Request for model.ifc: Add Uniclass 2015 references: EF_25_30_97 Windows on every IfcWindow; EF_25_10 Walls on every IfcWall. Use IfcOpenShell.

First a look at what the model holds.

```python
import ifcopenshell

model = ifcopenshell.open("model.ifc")
print(model.schema)
print("classifications:", [c.Name for c in model.by_type("IfcClassification")])
for ifc_class in ("IfcDoor", "IfcRoof", "IfcStair", "IfcWall", "IfcWindow"):
    print(ifc_class, len(model.by_type(ifc_class)))
```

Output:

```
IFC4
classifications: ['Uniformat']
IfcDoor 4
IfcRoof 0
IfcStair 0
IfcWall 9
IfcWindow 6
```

```python
import ifcopenshell
import ifcopenshell.api.classification

model = ifcopenshell.open("model.ifc")

system = ifcopenshell.api.classification.add_classification(model, classification="Uniclass 2015")

codes = {
    "IfcWindow": ("EF_25_30_97", "Windows"),
    "IfcWall": ("EF_25_10", "Walls"),
}
for ifc_class, (code, name) in codes.items():
    products = model.by_type(ifc_class)
    ifcopenshell.api.classification.add_reference(
        model, products=products, classification=system, identification=code, name=name
    )
    print(code, len(products))

model.write("model-out.ifc")
```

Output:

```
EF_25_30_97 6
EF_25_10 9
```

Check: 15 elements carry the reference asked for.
